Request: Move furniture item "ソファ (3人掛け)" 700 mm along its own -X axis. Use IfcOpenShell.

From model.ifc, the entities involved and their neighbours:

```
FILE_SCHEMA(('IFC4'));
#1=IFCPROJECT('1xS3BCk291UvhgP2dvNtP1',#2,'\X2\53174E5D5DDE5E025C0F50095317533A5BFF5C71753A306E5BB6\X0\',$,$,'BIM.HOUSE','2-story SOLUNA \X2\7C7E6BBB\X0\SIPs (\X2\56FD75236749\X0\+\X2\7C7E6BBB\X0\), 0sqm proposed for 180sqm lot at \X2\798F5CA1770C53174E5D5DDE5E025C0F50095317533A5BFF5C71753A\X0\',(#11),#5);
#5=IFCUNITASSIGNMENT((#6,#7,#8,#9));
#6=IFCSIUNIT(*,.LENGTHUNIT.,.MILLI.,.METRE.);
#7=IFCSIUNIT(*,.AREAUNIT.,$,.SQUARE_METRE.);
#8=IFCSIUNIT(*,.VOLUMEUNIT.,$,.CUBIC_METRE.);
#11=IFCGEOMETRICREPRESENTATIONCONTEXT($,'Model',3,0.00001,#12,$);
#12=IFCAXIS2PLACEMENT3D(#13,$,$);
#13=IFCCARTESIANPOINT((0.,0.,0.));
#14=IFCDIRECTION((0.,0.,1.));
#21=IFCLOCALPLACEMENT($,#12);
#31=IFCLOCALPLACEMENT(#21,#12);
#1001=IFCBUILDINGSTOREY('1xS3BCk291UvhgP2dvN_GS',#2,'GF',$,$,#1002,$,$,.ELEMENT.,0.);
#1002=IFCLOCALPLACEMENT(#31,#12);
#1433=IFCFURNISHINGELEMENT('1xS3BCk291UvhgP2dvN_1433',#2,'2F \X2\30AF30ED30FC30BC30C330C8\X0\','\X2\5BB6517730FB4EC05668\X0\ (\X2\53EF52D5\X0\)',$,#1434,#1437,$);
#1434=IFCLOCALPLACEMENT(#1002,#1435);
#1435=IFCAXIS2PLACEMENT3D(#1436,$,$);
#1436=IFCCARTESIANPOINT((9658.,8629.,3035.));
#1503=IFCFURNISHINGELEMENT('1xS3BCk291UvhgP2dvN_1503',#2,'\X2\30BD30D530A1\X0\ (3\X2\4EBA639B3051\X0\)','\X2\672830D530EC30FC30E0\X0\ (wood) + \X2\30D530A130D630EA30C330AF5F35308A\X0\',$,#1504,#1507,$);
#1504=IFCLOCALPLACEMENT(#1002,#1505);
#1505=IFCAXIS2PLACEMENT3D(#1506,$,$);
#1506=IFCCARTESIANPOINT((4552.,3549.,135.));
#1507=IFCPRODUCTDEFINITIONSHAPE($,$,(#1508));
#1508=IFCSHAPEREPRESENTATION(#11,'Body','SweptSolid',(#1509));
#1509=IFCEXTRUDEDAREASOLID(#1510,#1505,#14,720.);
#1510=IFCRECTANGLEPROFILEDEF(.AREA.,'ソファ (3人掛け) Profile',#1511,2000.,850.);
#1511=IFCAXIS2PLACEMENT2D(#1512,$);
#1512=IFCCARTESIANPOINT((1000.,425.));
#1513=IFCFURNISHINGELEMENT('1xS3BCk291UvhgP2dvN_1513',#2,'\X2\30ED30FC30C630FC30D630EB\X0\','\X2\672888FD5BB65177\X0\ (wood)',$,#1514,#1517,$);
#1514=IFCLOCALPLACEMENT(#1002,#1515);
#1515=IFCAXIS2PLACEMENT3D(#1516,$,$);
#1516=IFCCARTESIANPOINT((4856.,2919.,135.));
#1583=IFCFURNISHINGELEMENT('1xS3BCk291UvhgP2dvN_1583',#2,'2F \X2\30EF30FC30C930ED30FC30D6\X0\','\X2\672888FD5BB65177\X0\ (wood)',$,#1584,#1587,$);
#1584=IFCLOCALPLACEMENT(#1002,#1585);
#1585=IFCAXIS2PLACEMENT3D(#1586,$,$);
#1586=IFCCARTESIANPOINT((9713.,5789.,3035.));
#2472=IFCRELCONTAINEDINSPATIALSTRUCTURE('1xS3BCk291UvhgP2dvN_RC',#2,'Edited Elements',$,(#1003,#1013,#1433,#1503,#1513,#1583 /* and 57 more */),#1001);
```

```python
import ifcopenshell
import ifcopenshell.api.geometry
import ifcopenshell.util.placement
import ifcopenshell.util.unit

model = ifcopenshell.open("model.ifc")
unit_scale = ifcopenshell.util.unit.calculate_unit_scale(model)

item = model.by_guid("1xS3BCk291UvhgP2dvN_1503")
matrix = ifcopenshell.util.placement.get_local_placement(item.ObjectPlacement)
matrix[:3, 3] -= matrix[:3, 0] * 0.7 / unit_scale
ifcopenshell.api.geometry.edit_object_placement(model, product=item, matrix=matrix, is_si=False)

print(ifcopenshell.util.placement.get_local_placement(item.ObjectPlacement).round(3) + 0.0)

model.write("model_updated.ifc")
```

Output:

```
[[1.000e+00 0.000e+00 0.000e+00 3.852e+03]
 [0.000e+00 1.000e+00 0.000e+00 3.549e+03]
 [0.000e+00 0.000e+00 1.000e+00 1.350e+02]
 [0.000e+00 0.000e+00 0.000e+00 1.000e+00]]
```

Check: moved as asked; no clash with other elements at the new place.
